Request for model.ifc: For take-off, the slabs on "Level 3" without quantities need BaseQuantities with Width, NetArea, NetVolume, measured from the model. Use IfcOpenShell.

First a look at what the model holds.

```python
import ifcopenshell
import ifcopenshell.util.element
import ifcopenshell.util.unit

model = ifcopenshell.open("model.ifc")
print(model.schema)
for unit_type in ("LENGTHUNIT", "AREAUNIT", "VOLUMEUNIT"):
    print(unit_type, ifcopenshell.util.unit.calculate_unit_scale(model, unit_type))
storey = next(s for s in model.by_type("IfcBuildingStorey") if s.Name == "Level 3")
slabs = [e for e in ifcopenshell.util.element.get_decomposition(storey) if e.is_a("IfcSlab")]
for e in sorted(slabs, key=lambda e: e.id()):
    print(e.id(), e.is_a(), e.Name, list(ifcopenshell.util.element.get_psets(e, qtos_only=True)), sep=" | ")
```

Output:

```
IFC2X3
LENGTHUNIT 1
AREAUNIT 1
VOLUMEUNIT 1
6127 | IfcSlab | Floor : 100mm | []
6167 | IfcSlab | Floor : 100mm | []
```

```python
import ifcopenshell
import ifcopenshell.api.pset
import ifcopenshell.geom
import ifcopenshell.util.element
import ifcopenshell.util.shape
import ifcopenshell.util.unit

model = ifcopenshell.open("model.ifc")
unit_scale = ifcopenshell.util.unit.calculate_unit_scale(model)
area_scale = ifcopenshell.util.unit.calculate_unit_scale(model, "AREAUNIT")
volume_scale = ifcopenshell.util.unit.calculate_unit_scale(model, "VOLUMEUNIT")
settings = ifcopenshell.geom.settings()

storey = next(s for s in model.by_type("IfcBuildingStorey") if s.Name == "Level 3")
slabs = [e for e in ifcopenshell.util.element.get_decomposition(storey) if e.is_a("IfcSlab")]

for e in sorted(slabs, key=lambda e: e.id()):
    if ifcopenshell.util.element.get_psets(e, qtos_only=True, should_inherit=False):
        continue
    # Geometry comes back in metres, in the element's own axes.
    shape = ifcopenshell.geom.create_shape(settings, e)
    values = {
        "Width": ifcopenshell.util.shape.get_z(shape.geometry) / unit_scale,
        "NetArea": ifcopenshell.util.shape.get_footprint_area(shape.geometry) / area_scale,
        "NetVolume": ifcopenshell.util.shape.get_volume(shape.geometry) / volume_scale,
    }
    qto = ifcopenshell.api.pset.add_qto(model, product=e, name="BaseQuantities")
    ifcopenshell.api.pset.edit_qto(model, qto=qto, properties=values)
    print(e.id(), {k: round(v, 3) for k, v in values.items()})

model.write("model_rev.ifc")
```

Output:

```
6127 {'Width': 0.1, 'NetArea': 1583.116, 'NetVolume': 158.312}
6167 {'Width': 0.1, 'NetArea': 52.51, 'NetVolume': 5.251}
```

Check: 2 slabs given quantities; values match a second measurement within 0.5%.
